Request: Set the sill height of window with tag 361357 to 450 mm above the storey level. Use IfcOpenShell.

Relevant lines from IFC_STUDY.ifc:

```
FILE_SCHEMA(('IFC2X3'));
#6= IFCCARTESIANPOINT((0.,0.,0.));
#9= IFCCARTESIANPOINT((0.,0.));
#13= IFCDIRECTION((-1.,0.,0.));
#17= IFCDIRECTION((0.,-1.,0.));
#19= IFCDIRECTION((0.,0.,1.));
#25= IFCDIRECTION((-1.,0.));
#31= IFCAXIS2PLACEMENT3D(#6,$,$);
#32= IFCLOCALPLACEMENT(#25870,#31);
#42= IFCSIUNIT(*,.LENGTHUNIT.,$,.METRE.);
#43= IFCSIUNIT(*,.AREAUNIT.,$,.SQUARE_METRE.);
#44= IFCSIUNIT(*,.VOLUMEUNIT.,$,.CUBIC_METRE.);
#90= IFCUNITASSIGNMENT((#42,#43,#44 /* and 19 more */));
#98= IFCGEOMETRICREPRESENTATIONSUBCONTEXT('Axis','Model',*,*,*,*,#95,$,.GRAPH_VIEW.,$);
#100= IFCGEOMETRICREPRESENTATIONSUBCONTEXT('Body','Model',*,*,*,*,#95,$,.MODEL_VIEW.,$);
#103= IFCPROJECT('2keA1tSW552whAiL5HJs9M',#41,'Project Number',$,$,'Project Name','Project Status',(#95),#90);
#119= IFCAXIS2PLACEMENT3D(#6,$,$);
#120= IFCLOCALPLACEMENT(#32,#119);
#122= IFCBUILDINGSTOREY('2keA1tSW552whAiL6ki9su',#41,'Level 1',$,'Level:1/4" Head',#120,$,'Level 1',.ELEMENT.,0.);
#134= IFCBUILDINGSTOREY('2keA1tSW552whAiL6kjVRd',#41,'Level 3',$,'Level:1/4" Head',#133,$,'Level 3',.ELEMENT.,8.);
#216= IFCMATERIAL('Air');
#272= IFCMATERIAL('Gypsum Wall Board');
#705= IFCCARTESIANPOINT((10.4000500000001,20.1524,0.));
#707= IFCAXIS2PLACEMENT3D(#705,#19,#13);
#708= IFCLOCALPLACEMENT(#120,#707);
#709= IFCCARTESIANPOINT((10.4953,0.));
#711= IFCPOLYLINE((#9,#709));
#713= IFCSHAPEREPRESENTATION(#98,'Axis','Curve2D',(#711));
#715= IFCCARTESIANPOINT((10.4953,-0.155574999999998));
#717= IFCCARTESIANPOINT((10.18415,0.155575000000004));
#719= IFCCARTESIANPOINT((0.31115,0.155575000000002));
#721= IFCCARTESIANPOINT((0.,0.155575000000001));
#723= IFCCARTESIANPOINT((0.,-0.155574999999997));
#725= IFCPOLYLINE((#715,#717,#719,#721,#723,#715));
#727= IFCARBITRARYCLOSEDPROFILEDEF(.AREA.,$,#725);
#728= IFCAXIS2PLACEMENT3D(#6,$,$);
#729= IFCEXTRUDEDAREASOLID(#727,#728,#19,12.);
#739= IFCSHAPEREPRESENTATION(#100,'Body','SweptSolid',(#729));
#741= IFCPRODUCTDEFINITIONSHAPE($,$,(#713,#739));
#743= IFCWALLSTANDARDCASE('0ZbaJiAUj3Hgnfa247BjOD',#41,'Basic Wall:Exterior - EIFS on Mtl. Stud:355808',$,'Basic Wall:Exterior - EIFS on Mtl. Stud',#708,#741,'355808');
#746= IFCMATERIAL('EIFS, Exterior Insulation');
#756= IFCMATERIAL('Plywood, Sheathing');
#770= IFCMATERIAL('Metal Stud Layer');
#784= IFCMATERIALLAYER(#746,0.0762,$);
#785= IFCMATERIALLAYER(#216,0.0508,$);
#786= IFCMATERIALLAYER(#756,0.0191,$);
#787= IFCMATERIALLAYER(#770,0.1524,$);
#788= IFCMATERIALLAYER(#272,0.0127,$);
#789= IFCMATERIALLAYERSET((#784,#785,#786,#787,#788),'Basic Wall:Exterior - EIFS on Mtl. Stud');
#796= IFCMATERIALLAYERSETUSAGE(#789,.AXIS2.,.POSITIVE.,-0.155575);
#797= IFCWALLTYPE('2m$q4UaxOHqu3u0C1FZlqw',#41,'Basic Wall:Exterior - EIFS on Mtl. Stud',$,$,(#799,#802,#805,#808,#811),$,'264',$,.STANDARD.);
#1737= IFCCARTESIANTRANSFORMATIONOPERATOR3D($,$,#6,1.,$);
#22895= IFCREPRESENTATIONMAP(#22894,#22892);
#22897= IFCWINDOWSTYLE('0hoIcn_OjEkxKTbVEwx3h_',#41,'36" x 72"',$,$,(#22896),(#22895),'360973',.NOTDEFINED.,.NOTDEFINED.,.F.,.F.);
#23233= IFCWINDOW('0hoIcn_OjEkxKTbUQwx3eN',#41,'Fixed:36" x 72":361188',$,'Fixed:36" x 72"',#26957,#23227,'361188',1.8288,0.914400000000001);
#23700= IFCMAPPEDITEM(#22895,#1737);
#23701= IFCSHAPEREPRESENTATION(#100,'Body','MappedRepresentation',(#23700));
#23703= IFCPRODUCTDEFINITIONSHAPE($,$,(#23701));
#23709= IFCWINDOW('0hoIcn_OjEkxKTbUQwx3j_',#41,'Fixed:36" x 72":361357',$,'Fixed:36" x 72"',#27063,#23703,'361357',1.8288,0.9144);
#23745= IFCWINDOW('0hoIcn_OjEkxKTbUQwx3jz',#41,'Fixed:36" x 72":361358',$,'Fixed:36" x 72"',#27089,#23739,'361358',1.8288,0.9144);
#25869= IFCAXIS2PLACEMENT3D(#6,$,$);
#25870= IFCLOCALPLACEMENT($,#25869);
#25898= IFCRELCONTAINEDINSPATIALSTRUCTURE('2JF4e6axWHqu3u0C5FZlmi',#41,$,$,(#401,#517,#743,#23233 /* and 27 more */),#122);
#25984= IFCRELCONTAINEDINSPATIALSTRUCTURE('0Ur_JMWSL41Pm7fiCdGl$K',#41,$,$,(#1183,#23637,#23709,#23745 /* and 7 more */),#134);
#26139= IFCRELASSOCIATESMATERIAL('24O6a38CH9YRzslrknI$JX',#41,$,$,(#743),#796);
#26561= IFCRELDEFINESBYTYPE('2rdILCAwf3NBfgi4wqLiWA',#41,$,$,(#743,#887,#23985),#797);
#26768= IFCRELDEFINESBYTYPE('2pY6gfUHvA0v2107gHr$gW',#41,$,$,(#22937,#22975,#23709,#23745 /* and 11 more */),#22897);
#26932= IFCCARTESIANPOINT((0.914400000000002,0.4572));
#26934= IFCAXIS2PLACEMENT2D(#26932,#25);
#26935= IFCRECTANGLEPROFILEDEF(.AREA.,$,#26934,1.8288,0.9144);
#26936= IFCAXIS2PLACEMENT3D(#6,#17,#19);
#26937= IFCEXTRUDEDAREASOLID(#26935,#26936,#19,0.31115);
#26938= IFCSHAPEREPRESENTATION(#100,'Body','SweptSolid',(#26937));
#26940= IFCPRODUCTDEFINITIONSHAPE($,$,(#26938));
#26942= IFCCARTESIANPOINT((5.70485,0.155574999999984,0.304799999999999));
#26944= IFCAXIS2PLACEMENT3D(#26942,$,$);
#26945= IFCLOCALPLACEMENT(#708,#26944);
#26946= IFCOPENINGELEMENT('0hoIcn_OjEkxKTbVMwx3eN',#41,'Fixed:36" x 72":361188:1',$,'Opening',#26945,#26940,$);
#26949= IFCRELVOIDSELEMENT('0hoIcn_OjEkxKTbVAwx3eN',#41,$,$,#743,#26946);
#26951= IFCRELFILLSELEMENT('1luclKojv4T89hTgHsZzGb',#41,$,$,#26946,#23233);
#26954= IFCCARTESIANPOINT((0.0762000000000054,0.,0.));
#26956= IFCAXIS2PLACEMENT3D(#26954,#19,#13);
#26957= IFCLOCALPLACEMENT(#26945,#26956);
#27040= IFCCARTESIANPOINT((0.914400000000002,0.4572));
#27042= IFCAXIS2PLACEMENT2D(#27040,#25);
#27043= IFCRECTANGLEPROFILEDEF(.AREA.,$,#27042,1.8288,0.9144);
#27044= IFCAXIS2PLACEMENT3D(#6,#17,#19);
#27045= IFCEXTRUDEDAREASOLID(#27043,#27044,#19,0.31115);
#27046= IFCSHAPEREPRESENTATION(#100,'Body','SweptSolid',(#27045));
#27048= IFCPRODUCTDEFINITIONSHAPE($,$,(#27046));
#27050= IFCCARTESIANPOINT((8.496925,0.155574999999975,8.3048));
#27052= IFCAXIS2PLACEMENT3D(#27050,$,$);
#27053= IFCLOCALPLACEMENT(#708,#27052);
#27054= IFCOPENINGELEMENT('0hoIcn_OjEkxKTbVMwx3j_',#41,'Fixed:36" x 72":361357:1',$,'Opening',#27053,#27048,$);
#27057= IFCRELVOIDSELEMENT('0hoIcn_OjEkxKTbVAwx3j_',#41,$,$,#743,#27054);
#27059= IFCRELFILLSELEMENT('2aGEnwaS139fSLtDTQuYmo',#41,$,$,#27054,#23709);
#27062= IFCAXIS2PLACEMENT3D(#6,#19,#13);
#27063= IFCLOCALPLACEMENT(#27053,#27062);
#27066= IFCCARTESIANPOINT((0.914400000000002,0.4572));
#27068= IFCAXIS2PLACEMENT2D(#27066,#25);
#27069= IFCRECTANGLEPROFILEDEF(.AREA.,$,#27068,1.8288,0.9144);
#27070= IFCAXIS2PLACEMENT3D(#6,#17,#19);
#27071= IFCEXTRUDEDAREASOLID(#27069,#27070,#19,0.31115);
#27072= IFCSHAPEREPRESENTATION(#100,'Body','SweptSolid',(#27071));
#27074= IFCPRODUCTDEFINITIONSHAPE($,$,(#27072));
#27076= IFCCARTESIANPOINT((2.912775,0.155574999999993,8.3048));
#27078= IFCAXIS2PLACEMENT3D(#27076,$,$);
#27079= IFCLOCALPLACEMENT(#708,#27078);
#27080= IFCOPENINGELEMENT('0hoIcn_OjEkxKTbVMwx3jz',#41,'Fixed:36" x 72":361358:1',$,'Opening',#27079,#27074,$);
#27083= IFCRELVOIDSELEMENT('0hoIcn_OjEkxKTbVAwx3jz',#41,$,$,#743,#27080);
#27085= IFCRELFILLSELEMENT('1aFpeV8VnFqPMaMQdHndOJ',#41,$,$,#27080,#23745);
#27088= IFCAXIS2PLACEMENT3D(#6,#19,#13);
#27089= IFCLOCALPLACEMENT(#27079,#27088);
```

```python
import numpy as np
import ifcopenshell
import ifcopenshell.api.geometry
import ifcopenshell.geom
import ifcopenshell.util.element
import ifcopenshell.util.placement
import ifcopenshell.util.shape
import ifcopenshell.util.unit

model = ifcopenshell.open("IFC_STUDY.ifc")
unit_scale = ifcopenshell.util.unit.calculate_unit_scale(model)

window = model.by_guid("0hoIcn_OjEkxKTbUQwx3j_")
opening = window.FillsVoids[0].RelatingOpeningElement
storey = ifcopenshell.util.element.get_container(window, ifc_class="IfcBuildingStorey")
level = ifcopenshell.util.placement.get_local_placement(storey.ObjectPlacement)[2, 3]

# The opening's origin need not be at the sill, so measure its lowest point.
shape = ifcopenshell.geom.create_shape(ifcopenshell.geom.settings(), opening)
bottom = ifcopenshell.util.shape.get_shape_bottom_elevation(shape, shape.geometry) / unit_scale
dz = level + 0.45 - bottom

shift = np.array([0.0, 0.0, dz])
# The window is placed relative to its opening, so it follows when the opening moves.
matrix = ifcopenshell.util.placement.get_local_placement(opening.ObjectPlacement)
matrix[:3, 3] += shift
ifcopenshell.api.geometry.edit_object_placement(
    model, product=opening, matrix=matrix, is_si=False, should_transform_children=True
)

print(f"moved by {dz * unit_scale:+.3f} m")

model.write("IFC_STUDY-out.ifc")
```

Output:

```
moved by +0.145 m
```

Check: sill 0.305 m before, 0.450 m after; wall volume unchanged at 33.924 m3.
